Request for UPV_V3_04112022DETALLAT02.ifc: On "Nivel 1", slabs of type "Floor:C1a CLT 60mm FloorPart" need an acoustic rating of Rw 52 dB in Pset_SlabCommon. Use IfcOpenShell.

First a look at what the model holds.

```python
import ifcopenshell
import ifcopenshell.util.element

model = ifcopenshell.open("UPV_V3_04112022DETALLAT02.ifc")
print(model.schema)
storey = next(s for s in model.by_type("IfcBuildingStorey") if s.Name == "Nivel 1")
slabs = [e for e in ifcopenshell.util.element.get_decomposition(storey) if e.is_a("IfcSlab")]
seen = {}
for e in slabs:
    element_type = ifcopenshell.util.element.get_type(e)
    key = (element_type.Name if element_type != e and element_type else None, ifcopenshell.util.element.get_pset(e, "Pset_SlabCommon", "AcousticRating"))
    seen[key] = seen.get(key, 0) + 1
for (name, value), count in sorted(seen.items(), key=str):
    print(count, "x", name, "|", value)
```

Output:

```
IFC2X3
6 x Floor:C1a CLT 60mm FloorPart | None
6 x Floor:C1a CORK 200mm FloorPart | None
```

```python
import ifcopenshell
import ifcopenshell.api.pset
import ifcopenshell.util.element

model = ifcopenshell.open("UPV_V3_04112022DETALLAT02.ifc")

storey = next(s for s in model.by_type("IfcBuildingStorey") if s.Name == "Nivel 1")
slabs = [e for e in ifcopenshell.util.element.get_decomposition(storey) if e.is_a("IfcSlab")]

count = 0
for e in slabs:
    element_type = ifcopenshell.util.element.get_type(e)
    if element_type in (None, e) or element_type.Name != "Floor:C1a CLT 60mm FloorPart":
        continue
    # add_pset returns the element's existing set when there is one.
    pset = ifcopenshell.api.pset.add_pset(model, product=e, name="Pset_SlabCommon")
    ifcopenshell.api.pset.edit_pset(model, pset=pset, properties={"AcousticRating": "Rw 52 dB"})
    count += 1

print(count, "slabs updated")

model.write("UPV_V3_04112022DETALLAT02_updated.ifc")
```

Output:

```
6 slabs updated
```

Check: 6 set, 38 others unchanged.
